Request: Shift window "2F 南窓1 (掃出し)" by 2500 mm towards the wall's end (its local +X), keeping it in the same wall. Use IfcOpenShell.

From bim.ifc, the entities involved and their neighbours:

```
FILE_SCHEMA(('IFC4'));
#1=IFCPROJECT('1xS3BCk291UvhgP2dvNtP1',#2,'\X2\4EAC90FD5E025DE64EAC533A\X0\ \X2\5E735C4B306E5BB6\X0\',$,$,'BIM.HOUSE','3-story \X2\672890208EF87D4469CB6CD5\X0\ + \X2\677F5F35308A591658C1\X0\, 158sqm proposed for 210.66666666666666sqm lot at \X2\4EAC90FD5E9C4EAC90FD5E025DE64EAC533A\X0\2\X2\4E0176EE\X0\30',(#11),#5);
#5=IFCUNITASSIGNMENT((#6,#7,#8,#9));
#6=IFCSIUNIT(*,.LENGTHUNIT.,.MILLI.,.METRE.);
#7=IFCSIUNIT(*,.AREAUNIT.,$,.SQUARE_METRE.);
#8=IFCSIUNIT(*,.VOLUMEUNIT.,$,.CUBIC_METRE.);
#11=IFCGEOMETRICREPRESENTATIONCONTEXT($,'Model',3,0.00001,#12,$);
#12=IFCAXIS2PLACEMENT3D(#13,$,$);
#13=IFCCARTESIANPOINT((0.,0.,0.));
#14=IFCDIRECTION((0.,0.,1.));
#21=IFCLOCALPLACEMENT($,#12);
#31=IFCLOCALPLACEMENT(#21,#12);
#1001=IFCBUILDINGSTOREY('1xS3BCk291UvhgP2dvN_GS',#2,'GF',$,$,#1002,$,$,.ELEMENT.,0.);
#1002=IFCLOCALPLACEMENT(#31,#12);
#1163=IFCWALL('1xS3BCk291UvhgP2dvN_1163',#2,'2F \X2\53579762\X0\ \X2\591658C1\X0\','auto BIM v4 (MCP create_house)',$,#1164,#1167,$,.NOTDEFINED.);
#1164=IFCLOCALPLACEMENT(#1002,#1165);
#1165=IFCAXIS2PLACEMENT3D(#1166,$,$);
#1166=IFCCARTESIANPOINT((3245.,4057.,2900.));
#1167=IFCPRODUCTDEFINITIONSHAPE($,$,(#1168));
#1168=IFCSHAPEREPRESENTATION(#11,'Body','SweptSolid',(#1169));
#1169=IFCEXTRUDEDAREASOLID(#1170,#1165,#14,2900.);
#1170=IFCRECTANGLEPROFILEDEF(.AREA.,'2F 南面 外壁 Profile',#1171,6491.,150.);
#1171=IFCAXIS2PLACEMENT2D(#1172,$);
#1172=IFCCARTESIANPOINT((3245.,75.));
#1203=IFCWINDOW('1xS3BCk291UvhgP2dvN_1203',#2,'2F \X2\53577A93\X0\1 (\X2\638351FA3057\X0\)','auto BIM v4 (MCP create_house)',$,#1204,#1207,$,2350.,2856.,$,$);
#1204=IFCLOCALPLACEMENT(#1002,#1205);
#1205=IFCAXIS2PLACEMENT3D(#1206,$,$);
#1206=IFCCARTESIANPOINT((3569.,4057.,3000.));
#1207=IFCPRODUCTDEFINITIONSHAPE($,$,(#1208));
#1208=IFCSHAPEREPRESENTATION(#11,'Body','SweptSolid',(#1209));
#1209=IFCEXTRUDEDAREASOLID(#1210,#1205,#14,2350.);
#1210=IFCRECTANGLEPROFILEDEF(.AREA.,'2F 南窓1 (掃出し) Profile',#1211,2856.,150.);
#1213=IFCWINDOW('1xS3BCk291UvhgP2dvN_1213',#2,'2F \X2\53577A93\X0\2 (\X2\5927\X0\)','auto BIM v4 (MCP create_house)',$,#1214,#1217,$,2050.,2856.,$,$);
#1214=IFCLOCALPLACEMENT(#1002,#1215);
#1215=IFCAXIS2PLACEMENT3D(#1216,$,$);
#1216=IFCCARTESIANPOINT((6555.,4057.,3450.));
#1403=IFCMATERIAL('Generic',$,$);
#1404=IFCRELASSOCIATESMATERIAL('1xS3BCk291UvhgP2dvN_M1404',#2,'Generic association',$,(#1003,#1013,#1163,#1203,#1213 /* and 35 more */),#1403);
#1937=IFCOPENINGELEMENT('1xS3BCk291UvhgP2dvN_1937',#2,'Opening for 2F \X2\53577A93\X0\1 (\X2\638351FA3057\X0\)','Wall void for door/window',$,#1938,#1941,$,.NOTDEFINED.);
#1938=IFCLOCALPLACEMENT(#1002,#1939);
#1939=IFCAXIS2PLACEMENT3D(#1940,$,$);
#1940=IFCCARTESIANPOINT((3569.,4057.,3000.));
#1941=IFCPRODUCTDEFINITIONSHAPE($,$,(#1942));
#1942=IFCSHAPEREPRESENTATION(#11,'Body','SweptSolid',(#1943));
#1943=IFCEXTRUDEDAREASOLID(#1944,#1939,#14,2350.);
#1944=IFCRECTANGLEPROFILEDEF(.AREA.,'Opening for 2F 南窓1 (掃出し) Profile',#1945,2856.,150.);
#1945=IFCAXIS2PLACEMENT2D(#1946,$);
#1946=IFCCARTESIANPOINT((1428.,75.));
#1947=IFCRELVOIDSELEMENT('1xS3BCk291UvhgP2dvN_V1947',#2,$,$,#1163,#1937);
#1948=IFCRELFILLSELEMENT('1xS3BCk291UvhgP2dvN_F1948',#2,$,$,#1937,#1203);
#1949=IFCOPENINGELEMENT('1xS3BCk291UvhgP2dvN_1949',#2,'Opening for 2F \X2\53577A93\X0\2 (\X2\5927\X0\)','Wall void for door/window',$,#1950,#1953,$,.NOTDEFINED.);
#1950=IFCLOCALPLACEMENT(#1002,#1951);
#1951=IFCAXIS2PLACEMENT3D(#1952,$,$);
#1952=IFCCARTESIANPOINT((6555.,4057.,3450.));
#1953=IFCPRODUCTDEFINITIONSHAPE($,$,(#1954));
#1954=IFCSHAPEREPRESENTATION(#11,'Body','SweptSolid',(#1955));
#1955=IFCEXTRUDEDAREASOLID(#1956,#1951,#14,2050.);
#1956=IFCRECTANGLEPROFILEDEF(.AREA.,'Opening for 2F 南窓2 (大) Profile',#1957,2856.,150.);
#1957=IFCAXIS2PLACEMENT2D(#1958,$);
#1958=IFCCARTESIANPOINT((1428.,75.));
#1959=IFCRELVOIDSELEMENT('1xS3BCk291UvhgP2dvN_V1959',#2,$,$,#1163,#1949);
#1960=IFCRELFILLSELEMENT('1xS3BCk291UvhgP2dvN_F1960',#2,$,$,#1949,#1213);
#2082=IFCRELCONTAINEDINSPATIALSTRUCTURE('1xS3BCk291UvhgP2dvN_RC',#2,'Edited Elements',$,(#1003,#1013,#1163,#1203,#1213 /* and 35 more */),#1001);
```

```python
import ifcopenshell
import ifcopenshell.api.geometry
import ifcopenshell.util.placement
import ifcopenshell.util.unit

model = ifcopenshell.open("bim.ifc")
unit_scale = ifcopenshell.util.unit.calculate_unit_scale(model)

window = model.by_guid("1xS3BCk291UvhgP2dvN_1203")
opening = window.FillsVoids[0].RelatingOpeningElement
wall = opening.VoidsElements[0].RelatingBuildingElement

wall_matrix = ifcopenshell.util.placement.get_local_placement(wall.ObjectPlacement)
shift = wall_matrix[:3, 0] * 2.5 / unit_scale
before = ifcopenshell.util.placement.get_local_placement(window.ObjectPlacement)[:3, 3].copy()

# The window is not placed relative to its opening, so move both.
for product in (opening, window):
    matrix = ifcopenshell.util.placement.get_local_placement(product.ObjectPlacement)
    matrix[:3, 3] += shift
    ifcopenshell.api.geometry.edit_object_placement(model, product=product, matrix=matrix, is_si=False)

after = ifcopenshell.util.placement.get_local_placement(window.ObjectPlacement)[:3, 3]
print("window moved by", (after - before).round(3) + 0.0)

model.write("bim_rev.ifc")
```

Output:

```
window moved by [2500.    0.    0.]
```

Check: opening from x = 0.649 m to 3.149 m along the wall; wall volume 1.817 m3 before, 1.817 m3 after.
